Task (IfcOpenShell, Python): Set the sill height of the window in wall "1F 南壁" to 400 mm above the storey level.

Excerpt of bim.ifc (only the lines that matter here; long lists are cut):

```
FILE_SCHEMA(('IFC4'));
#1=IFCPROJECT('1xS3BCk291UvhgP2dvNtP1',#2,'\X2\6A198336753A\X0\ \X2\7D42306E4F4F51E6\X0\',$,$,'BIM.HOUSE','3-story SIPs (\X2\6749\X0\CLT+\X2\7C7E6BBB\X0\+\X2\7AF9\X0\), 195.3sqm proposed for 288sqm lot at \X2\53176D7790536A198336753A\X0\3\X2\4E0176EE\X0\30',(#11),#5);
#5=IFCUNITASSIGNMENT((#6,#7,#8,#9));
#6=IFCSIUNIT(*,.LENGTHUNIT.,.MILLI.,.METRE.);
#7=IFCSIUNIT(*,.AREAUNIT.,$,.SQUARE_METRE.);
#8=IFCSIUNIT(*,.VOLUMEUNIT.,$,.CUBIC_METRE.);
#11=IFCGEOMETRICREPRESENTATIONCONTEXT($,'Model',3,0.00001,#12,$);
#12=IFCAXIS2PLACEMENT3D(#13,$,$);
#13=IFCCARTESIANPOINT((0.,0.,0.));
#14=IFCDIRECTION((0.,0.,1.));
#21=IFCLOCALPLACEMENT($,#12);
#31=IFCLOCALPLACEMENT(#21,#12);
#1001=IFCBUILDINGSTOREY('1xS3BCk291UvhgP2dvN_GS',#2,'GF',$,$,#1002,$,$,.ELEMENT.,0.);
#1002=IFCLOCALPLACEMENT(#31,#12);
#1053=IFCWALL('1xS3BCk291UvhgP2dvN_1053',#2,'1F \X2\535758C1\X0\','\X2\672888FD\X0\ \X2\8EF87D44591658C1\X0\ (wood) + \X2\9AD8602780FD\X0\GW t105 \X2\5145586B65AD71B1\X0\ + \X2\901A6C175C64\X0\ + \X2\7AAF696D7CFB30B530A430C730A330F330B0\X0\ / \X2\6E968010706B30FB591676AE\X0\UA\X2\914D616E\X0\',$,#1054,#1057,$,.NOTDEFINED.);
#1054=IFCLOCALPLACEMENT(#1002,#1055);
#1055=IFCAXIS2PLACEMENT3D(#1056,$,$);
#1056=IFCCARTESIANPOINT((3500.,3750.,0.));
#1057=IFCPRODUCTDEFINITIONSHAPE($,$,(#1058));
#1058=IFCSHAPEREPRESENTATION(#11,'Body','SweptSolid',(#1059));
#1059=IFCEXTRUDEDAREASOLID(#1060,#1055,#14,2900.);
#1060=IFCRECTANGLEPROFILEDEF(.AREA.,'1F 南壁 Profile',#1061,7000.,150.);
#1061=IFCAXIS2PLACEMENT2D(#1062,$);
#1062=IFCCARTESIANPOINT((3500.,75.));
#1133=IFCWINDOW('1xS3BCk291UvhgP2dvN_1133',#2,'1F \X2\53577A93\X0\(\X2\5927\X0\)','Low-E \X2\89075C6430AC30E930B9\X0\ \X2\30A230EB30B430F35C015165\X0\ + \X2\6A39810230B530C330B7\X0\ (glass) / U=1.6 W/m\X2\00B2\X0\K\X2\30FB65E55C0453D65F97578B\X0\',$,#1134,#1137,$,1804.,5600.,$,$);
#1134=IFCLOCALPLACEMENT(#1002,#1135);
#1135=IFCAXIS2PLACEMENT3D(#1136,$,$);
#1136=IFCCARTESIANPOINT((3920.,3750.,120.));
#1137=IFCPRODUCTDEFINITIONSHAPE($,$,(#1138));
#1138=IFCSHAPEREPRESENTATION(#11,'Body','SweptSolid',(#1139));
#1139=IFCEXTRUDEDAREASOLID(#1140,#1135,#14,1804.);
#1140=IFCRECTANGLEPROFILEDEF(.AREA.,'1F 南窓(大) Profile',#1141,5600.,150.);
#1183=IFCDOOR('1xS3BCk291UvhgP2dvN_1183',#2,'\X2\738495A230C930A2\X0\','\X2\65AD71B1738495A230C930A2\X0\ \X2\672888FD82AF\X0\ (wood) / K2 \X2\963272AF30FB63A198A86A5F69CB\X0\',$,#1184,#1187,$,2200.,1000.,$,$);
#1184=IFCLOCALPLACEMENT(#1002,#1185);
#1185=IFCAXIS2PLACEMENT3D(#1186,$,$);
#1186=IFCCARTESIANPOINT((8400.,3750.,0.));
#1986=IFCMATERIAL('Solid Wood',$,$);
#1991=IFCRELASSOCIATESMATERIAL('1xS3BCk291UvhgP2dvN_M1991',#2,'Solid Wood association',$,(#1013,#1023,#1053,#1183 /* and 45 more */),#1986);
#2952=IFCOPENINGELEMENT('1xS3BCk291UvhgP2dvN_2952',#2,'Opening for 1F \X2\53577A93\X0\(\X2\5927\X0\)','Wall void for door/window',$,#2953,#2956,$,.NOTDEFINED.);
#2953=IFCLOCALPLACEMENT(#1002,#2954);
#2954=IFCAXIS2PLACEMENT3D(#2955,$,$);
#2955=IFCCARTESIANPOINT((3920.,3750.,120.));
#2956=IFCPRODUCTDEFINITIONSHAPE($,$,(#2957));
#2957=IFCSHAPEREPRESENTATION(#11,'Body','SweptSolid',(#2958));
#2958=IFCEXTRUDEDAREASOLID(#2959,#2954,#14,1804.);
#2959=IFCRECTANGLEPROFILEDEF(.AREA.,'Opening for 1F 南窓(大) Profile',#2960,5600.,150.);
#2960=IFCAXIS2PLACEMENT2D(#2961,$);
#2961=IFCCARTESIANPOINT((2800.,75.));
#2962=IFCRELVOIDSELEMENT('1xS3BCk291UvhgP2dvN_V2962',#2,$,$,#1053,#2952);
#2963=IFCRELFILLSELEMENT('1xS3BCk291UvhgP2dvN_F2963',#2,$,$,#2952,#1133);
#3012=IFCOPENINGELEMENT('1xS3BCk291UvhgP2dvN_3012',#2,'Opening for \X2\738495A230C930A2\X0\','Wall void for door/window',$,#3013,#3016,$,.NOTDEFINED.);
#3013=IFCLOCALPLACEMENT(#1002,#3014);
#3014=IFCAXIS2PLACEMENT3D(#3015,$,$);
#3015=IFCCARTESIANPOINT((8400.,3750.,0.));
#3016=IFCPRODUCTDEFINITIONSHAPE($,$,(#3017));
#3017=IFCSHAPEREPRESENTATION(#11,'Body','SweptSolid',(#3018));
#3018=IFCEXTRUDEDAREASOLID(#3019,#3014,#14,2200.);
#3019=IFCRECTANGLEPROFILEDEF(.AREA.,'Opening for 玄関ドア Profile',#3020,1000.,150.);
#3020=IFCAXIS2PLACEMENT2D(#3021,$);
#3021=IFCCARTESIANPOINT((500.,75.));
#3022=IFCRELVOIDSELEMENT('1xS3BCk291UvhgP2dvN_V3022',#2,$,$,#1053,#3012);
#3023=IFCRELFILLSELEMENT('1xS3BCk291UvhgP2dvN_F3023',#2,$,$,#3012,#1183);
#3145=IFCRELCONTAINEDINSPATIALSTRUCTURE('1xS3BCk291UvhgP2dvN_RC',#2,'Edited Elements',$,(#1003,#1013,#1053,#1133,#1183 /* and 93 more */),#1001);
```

```python
import numpy as np
import ifcopenshell
import ifcopenshell.api.geometry
import ifcopenshell.geom
import ifcopenshell.util.element
import ifcopenshell.util.placement
import ifcopenshell.util.shape
import ifcopenshell.util.unit

model = ifcopenshell.open("bim.ifc")
unit_scale = ifcopenshell.util.unit.calculate_unit_scale(model)

window = model.by_guid("1xS3BCk291UvhgP2dvN_1133")
opening = window.FillsVoids[0].RelatingOpeningElement
storey = ifcopenshell.util.element.get_container(window, ifc_class="IfcBuildingStorey")
level = ifcopenshell.util.placement.get_local_placement(storey.ObjectPlacement)[2, 3]

# The opening's origin need not be at the sill, so measure its lowest point.
shape = ifcopenshell.geom.create_shape(ifcopenshell.geom.settings(), opening)
bottom = ifcopenshell.util.shape.get_shape_bottom_elevation(shape, shape.geometry) / unit_scale
dz = level + 400.0 - bottom

shift = np.array([0.0, 0.0, dz])
# The window is not placed relative to its opening, so move both.
for product in (opening, window):
    matrix = ifcopenshell.util.placement.get_local_placement(product.ObjectPlacement)
    matrix[:3, 3] += shift
    ifcopenshell.api.geometry.edit_object_placement(model, product=product, matrix=matrix, is_si=False)

print(f"moved by {dz * unit_scale:+.3f} m")

model.write("bim_updated.ifc")
```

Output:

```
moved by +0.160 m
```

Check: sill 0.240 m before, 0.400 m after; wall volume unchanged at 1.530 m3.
